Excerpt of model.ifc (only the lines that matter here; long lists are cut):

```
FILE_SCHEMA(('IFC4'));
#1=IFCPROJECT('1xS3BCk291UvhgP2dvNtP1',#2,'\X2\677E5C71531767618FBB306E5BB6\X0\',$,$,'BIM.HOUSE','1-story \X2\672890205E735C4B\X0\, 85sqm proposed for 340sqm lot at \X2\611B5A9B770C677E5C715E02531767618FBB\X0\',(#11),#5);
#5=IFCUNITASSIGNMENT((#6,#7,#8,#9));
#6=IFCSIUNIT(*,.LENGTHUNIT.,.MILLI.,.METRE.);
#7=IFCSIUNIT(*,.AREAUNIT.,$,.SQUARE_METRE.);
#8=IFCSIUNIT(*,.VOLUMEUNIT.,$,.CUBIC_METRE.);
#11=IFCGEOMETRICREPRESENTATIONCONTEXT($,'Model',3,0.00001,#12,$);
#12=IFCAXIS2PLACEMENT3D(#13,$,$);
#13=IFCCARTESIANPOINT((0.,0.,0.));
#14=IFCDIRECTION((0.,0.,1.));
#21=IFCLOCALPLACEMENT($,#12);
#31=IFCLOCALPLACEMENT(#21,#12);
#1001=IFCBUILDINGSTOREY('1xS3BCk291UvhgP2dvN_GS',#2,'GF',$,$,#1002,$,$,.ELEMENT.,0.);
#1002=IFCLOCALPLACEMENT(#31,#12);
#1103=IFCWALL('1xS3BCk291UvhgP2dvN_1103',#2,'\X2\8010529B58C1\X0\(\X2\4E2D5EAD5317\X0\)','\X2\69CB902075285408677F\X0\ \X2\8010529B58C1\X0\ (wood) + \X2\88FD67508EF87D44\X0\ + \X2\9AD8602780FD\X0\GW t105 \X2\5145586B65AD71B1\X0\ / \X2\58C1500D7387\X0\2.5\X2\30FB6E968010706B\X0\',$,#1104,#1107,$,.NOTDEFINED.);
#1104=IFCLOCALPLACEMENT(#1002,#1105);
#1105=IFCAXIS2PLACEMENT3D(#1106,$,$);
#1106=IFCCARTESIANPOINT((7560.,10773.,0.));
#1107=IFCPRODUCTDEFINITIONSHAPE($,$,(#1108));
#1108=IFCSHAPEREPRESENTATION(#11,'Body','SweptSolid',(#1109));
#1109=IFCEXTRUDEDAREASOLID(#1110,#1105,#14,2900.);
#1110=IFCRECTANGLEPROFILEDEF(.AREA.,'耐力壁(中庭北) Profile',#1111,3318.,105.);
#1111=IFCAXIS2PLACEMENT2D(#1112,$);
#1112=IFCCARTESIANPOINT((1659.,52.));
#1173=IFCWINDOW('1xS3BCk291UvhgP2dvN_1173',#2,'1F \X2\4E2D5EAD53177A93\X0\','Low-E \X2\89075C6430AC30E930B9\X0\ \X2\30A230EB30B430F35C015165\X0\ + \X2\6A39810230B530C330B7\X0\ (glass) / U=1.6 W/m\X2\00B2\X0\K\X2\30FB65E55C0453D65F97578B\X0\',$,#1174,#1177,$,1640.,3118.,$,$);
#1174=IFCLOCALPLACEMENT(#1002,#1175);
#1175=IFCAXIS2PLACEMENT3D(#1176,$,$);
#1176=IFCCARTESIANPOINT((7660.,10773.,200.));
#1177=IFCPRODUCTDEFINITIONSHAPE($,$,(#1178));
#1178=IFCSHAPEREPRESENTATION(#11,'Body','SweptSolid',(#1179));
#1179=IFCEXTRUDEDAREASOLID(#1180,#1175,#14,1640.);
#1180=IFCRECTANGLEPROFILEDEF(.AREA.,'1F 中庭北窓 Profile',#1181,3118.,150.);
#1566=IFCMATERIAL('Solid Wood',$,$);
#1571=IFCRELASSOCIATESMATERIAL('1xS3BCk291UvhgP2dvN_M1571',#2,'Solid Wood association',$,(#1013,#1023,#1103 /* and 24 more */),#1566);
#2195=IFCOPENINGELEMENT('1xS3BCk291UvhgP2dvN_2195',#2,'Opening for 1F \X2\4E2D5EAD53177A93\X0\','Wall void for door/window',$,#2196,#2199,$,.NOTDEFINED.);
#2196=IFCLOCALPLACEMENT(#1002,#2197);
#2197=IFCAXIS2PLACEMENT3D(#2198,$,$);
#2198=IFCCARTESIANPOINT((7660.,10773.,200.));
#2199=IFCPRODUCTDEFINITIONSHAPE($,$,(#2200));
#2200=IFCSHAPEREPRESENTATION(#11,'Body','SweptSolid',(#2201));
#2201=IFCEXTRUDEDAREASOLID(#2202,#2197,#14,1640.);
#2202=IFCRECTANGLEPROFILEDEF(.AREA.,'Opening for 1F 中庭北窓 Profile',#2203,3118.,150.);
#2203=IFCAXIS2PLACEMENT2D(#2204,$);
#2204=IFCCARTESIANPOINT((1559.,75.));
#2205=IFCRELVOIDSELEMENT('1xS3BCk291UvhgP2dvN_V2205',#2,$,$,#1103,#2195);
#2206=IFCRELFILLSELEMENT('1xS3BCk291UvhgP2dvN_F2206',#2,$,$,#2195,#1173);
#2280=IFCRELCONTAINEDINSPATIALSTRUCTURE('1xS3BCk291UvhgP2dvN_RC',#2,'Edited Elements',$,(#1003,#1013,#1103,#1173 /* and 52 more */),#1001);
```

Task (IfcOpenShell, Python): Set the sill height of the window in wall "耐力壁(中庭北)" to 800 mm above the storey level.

```python
import numpy as np
import ifcopenshell
import ifcopenshell.api.geometry
import ifcopenshell.geom
import ifcopenshell.util.element
import ifcopenshell.util.placement
import ifcopenshell.util.shape
import ifcopenshell.util.unit

model = ifcopenshell.open("model.ifc")
unit_scale = ifcopenshell.util.unit.calculate_unit_scale(model)

window = model.by_guid("1xS3BCk291UvhgP2dvN_1173")
opening = window.FillsVoids[0].RelatingOpeningElement
storey = ifcopenshell.util.element.get_container(window, ifc_class="IfcBuildingStorey")
level = ifcopenshell.util.placement.get_local_placement(storey.ObjectPlacement)[2, 3]

# The opening's origin need not be at the sill, so measure its lowest point.
shape = ifcopenshell.geom.create_shape(ifcopenshell.geom.settings(), opening)
bottom = ifcopenshell.util.shape.get_shape_bottom_elevation(shape, shape.geometry) / unit_scale
dz = level + 800.0 - bottom

shift = np.array([0.0, 0.0, dz])
# The window is not placed relative to its opening, so move both.
for product in (opening, window):
    matrix = ifcopenshell.util.placement.get_local_placement(product.ObjectPlacement)
    matrix[:3, 3] += shift
    ifcopenshell.api.geometry.edit_object_placement(model, product=product, matrix=matrix, is_si=False)

print(f"moved by {dz * unit_scale:+.3f} m")

model.write("model-out.ifc")
```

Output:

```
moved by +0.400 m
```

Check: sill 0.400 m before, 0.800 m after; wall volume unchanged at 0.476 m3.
